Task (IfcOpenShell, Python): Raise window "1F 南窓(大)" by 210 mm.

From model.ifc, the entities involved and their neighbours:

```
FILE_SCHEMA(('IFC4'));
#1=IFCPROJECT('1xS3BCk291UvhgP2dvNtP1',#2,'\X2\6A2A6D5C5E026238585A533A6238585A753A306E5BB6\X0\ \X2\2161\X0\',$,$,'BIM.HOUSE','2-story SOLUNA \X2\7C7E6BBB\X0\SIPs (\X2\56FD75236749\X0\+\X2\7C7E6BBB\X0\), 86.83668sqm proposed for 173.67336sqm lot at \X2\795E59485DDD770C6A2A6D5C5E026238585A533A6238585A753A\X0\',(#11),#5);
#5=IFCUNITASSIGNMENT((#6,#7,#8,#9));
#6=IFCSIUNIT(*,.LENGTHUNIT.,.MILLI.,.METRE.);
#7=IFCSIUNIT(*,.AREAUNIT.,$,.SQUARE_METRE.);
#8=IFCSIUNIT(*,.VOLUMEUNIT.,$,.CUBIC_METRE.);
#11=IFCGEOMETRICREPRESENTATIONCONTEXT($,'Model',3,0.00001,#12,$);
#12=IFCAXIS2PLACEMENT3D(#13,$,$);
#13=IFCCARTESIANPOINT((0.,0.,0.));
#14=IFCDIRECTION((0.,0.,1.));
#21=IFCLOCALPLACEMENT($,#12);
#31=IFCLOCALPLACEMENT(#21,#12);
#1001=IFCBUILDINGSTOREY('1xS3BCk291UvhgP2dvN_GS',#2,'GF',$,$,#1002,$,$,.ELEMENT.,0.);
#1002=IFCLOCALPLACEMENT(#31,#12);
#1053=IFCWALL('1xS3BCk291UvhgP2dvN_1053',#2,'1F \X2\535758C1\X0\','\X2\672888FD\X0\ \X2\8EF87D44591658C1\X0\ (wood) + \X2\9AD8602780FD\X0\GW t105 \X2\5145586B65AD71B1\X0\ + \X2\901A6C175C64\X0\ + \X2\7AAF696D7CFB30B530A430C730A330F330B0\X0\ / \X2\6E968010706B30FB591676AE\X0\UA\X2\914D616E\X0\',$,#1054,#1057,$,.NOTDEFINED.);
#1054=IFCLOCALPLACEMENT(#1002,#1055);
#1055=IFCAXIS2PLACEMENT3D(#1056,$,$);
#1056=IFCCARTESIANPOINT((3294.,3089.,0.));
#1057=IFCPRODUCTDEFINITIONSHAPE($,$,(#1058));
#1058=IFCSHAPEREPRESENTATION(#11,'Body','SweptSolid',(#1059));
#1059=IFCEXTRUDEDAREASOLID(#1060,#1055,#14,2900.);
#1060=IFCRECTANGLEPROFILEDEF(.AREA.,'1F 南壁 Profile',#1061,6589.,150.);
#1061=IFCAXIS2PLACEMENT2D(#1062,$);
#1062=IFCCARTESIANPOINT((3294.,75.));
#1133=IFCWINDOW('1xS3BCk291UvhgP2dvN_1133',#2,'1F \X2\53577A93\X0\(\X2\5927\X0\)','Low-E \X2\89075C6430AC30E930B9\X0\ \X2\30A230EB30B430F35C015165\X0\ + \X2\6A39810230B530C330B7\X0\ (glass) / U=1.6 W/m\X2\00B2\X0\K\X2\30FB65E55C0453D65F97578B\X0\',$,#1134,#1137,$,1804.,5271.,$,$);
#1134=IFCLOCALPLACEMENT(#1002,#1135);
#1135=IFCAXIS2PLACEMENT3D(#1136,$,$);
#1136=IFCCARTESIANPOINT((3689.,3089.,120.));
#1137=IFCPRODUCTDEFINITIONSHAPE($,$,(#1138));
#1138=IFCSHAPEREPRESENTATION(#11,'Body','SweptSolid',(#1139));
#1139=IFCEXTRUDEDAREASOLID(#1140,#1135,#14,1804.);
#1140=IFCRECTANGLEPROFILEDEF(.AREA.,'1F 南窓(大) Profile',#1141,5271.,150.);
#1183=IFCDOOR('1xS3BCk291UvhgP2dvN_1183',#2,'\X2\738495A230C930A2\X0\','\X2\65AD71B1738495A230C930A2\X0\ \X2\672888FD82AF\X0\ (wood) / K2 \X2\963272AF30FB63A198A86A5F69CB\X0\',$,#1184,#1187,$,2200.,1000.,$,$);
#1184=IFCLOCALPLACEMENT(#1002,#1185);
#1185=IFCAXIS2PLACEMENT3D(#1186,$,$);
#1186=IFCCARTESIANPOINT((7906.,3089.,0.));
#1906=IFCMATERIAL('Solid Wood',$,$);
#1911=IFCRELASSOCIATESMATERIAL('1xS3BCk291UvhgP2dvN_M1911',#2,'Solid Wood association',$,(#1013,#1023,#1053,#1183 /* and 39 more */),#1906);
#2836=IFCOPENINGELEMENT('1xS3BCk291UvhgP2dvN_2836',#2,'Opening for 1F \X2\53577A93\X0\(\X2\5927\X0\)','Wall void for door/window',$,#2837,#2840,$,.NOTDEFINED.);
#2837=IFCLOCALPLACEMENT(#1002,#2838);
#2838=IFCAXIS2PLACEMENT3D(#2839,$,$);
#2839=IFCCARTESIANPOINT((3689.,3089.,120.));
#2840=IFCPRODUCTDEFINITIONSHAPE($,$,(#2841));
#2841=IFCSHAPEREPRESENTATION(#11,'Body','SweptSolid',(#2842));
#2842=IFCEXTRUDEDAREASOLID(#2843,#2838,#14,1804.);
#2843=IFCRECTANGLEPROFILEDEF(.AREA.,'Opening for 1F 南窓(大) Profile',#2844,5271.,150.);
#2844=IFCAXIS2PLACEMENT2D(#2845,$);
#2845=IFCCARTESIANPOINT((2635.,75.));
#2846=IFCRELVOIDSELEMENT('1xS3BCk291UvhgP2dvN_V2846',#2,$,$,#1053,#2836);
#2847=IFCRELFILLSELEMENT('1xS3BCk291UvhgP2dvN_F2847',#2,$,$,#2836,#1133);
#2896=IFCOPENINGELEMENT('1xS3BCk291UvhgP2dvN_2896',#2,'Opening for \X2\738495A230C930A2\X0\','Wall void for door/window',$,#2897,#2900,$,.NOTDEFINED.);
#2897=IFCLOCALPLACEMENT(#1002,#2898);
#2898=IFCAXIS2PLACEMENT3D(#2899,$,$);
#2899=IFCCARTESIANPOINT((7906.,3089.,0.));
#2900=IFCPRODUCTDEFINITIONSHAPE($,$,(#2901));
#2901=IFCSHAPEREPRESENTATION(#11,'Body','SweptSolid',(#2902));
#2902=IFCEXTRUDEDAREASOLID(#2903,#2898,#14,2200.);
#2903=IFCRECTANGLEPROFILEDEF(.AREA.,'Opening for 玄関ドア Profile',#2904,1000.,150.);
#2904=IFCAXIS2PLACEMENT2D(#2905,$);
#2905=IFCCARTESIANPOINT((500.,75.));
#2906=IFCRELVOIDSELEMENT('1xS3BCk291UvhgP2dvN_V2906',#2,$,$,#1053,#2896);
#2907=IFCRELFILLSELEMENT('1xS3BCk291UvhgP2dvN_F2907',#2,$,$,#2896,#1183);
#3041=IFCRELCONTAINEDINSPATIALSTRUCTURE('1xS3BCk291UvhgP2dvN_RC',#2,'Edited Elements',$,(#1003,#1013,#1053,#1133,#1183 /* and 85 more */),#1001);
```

```python
import numpy as np
import ifcopenshell
import ifcopenshell.api.geometry
import ifcopenshell.util.placement
import ifcopenshell.util.unit

model = ifcopenshell.open("model.ifc")
unit_scale = ifcopenshell.util.unit.calculate_unit_scale(model)

window = model.by_id(1133)
opening = window.FillsVoids[0].RelatingOpeningElement
dz = 210.0

shift = np.array([0.0, 0.0, dz])
# The window is not placed relative to its opening, so move both.
for product in (opening, window):
    matrix = ifcopenshell.util.placement.get_local_placement(product.ObjectPlacement)
    matrix[:3, 3] += shift
    ifcopenshell.api.geometry.edit_object_placement(model, product=product, matrix=matrix, is_si=False)

print(f"moved by {dz * unit_scale:+.3f} m")

model.write("model_rev.ifc")
```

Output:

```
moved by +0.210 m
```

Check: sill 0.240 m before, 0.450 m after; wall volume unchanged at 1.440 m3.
